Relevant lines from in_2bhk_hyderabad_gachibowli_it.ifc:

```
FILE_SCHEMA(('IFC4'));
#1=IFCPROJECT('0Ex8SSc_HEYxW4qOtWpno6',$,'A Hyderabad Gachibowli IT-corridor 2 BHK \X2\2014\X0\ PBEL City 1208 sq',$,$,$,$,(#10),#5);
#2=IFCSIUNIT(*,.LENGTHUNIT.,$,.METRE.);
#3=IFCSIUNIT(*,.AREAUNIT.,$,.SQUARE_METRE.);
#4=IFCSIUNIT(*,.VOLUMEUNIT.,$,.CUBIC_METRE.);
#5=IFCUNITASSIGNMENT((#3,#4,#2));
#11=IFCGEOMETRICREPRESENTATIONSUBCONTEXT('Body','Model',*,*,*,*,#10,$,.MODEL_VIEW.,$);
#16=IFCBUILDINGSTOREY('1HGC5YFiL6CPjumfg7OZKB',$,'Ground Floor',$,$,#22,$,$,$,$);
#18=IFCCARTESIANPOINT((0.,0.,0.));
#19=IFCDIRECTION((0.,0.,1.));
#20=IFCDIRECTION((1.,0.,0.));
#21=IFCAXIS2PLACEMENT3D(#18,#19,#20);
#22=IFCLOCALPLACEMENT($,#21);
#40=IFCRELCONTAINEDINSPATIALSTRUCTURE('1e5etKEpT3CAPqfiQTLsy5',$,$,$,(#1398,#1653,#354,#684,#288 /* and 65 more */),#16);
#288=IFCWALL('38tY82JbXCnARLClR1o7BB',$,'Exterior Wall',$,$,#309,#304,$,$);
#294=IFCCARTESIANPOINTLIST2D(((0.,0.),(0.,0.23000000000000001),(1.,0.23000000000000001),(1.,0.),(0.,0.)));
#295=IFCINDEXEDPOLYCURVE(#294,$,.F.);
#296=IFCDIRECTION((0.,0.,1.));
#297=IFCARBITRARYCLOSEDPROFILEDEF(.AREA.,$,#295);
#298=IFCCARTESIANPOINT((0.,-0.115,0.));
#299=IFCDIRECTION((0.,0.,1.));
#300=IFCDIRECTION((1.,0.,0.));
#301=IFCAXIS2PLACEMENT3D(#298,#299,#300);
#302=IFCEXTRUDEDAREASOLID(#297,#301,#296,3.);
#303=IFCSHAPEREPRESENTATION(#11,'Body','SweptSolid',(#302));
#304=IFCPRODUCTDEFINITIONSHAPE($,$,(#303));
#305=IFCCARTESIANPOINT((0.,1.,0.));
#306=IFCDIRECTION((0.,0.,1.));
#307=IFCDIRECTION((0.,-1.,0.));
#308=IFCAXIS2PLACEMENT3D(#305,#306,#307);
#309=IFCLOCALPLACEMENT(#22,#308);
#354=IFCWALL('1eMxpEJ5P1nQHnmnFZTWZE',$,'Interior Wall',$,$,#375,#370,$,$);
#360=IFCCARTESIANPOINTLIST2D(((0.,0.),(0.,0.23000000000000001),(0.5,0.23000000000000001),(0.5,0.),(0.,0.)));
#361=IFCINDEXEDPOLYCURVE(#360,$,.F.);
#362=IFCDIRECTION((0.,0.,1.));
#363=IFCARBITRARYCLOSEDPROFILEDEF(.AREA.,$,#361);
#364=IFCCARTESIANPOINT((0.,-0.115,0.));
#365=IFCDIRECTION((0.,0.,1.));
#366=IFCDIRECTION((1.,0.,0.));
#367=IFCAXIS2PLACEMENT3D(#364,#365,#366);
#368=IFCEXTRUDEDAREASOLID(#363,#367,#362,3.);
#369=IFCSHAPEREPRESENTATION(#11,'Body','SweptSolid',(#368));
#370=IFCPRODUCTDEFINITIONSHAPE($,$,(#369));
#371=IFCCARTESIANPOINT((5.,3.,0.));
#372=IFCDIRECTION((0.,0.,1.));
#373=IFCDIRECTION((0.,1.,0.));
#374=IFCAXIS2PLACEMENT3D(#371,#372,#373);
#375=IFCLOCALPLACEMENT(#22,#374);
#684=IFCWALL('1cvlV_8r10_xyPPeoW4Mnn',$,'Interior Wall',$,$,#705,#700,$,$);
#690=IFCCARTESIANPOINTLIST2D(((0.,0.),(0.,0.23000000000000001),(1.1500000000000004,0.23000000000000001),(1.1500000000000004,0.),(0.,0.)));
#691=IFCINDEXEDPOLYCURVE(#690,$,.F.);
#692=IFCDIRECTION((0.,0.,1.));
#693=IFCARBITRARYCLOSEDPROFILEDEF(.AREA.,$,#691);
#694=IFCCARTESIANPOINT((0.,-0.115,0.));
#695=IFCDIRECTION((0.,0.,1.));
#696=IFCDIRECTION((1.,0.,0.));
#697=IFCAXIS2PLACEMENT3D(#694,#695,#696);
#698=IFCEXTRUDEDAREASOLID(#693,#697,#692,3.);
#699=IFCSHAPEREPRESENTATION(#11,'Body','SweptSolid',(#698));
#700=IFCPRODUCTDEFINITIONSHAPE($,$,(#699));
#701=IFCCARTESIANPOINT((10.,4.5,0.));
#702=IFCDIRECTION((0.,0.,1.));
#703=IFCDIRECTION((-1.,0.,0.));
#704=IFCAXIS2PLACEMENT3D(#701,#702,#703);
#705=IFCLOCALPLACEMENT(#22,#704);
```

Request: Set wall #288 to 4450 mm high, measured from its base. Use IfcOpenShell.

```python
import ifcopenshell
import ifcopenshell.geom
import ifcopenshell.util.representation
import ifcopenshell.util.shape
import ifcopenshell.util.unit

model = ifcopenshell.open("in_2bhk_hyderabad_gachibowli_it.ifc")
unit_scale = ifcopenshell.util.unit.calculate_unit_scale(model)
settings = ifcopenshell.geom.settings()


def volume(element):
    """Net volume in cubic metres, openings subtracted."""
    shape = ifcopenshell.geom.create_shape(settings, element)
    return ifcopenshell.util.shape.get_volume(shape.geometry)


wall = model.by_guid("38tY82JbXCnARLClR1o7BB")
before = volume(wall)

body = ifcopenshell.util.representation.get_representation(wall, "Model", "Body")
solid = body.Items[0]
old_height = solid.Depth
solid.Depth = 4.45 / unit_scale
after = volume(wall)

print(f"height {old_height:g} -> {solid.Depth:g}, volume {before:.3f} -> {after:.3f} m3")

model.write("in_2bhk_hyderabad_gachibowli_it_rev.ifc")
```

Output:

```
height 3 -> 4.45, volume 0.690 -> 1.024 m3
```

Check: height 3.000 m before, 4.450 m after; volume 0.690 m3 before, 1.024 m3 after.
